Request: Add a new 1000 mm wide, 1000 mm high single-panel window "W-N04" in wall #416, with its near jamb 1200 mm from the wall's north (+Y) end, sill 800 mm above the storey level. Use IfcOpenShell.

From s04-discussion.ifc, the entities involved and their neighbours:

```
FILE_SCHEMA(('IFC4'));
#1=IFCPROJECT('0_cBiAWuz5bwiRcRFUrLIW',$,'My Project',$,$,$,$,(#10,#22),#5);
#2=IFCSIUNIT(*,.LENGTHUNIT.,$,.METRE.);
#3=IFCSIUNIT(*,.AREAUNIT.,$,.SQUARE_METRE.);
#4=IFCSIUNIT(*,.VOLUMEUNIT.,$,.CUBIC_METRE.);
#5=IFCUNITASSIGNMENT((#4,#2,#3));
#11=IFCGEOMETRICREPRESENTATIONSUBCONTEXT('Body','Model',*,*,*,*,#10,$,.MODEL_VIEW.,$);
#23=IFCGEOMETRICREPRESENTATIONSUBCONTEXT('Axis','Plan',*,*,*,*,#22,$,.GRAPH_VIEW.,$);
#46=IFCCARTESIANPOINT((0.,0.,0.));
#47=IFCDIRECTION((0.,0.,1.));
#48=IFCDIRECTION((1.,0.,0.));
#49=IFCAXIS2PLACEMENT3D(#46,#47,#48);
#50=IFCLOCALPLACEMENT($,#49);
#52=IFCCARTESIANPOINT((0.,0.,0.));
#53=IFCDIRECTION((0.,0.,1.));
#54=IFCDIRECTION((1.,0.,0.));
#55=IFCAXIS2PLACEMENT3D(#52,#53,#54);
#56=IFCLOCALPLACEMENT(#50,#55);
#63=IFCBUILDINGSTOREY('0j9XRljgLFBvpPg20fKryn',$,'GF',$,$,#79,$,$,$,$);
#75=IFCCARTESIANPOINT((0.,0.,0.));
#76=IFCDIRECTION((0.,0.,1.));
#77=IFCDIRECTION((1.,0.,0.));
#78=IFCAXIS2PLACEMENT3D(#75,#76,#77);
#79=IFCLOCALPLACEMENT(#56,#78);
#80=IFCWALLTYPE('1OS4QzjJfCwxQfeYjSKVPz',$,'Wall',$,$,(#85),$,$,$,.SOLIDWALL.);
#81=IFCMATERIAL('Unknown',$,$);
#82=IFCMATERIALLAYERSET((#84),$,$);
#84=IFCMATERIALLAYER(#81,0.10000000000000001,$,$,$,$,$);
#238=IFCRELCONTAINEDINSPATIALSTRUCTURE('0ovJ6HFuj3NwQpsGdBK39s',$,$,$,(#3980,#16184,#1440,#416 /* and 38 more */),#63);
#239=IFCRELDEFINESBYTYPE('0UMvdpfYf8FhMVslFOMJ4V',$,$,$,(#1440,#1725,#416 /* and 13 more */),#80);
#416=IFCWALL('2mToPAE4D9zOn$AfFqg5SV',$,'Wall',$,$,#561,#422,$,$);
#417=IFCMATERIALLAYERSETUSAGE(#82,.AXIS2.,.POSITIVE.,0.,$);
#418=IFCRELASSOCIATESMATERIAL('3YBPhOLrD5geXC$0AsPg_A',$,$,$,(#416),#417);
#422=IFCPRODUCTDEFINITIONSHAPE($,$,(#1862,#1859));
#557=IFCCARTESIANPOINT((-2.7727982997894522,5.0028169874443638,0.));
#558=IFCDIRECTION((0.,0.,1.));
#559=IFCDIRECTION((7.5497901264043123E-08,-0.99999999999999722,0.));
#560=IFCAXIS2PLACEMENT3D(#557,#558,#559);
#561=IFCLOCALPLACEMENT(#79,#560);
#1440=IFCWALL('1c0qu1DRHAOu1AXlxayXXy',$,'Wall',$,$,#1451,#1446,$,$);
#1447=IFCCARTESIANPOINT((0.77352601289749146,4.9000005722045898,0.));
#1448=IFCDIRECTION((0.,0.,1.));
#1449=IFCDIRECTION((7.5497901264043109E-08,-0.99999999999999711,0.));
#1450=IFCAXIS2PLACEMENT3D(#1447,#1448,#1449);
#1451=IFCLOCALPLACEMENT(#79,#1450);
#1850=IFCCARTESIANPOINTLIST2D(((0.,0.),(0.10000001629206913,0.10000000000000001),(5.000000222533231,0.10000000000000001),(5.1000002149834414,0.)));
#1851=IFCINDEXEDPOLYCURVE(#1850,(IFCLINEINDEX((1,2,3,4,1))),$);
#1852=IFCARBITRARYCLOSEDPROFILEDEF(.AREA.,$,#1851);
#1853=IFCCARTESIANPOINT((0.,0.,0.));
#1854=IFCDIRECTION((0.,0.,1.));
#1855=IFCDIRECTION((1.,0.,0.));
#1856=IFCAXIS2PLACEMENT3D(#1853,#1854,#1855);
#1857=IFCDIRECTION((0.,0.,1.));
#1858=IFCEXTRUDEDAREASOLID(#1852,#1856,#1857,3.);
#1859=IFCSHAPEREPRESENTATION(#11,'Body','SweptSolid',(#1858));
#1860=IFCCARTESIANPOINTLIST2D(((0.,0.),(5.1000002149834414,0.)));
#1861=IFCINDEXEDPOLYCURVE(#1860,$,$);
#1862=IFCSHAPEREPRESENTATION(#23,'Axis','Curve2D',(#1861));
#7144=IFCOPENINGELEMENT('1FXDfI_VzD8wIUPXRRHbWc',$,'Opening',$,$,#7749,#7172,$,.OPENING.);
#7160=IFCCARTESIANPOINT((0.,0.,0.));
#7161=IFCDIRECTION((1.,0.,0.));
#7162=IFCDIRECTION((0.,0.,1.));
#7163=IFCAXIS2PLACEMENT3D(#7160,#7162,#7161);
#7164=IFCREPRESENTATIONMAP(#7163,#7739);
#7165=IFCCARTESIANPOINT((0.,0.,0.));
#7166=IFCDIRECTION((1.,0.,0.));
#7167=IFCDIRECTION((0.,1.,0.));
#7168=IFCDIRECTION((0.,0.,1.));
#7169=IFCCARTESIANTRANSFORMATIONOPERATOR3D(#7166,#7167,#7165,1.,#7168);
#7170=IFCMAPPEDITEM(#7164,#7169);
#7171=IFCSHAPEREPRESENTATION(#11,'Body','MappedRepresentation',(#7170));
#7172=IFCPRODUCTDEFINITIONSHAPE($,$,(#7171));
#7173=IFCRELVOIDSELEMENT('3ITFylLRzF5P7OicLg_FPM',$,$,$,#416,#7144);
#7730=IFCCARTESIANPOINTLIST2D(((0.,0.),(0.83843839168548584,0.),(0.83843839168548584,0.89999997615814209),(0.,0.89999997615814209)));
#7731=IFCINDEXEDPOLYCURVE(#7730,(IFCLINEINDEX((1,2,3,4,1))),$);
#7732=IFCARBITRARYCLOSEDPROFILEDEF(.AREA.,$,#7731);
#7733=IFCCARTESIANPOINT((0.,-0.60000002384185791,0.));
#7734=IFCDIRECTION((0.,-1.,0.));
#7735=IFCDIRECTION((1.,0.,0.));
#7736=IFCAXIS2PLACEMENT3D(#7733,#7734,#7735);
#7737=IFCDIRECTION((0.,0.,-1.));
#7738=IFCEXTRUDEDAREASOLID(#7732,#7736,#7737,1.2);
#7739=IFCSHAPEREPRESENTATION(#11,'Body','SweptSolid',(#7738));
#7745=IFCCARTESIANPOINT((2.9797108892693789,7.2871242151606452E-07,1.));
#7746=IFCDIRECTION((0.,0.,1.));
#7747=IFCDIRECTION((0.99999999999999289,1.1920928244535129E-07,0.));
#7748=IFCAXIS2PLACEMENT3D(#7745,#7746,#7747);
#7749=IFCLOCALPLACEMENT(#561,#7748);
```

```python
import numpy as np
import ifcopenshell
import ifcopenshell.api.feature
import ifcopenshell.api.geometry
import ifcopenshell.api.root
import ifcopenshell.api.spatial
import ifcopenshell.geom
import ifcopenshell.util.element
import ifcopenshell.util.placement
import ifcopenshell.util.representation
import ifcopenshell.util.shape
import ifcopenshell.util.unit

model = ifcopenshell.open("s04-discussion.ifc")
unit_scale = ifcopenshell.util.unit.calculate_unit_scale(model)
settings = ifcopenshell.geom.settings()


def volume(element):
    """Net volume in cubic metres, openings subtracted."""
    shape = ifcopenshell.geom.create_shape(settings, element)
    return ifcopenshell.util.shape.get_volume(shape.geometry)


wall = model.by_guid("2mToPAE4D9zOn$AfFqg5SV")
storey = ifcopenshell.util.element.get_container(wall, ifc_class="IfcBuildingStorey")
context = ifcopenshell.util.representation.get_context(model, "Model", "Body", "MODEL_VIEW")
before = volume(wall)

width, height, from_end, sill = 1, 1, 1.2, 0.8  # metres

# The wall runs along its own X axis, and the end named is its -X end.
wall_shape = ifcopenshell.geom.create_shape(settings, wall)
x, y, z = ifcopenshell.util.shape.get_vertices(wall_shape.geometry).T
start = x.min() + from_end
face, thickness = float(y.min()), float(y.max() - y.min())
wall_matrix = ifcopenshell.util.placement.get_local_placement(wall.ObjectPlacement)
level = ifcopenshell.util.placement.get_local_placement(storey.ObjectPlacement)[2, 3]


def in_wall(x, y):
    """Placement at x, y metres in the wall's axes, at sill height."""
    matrix = wall_matrix.copy()
    matrix[:, 3] = wall_matrix @ np.array([x / unit_scale, y / unit_scale, 0.0, 1.0])
    matrix[2, 3] = level + sill / unit_scale
    return matrix


# Opening: a box that overshoots both wall faces by 50 mm.
opening = ifcopenshell.api.root.create_entity(model, ifc_class="IfcOpeningElement", predefined_type="OPENING")
box = ifcopenshell.api.geometry.add_wall_representation(
    model, context=context, length=width, height=height, thickness=thickness + 0.1
)
ifcopenshell.api.geometry.assign_representation(model, product=opening, representation=box)
ifcopenshell.api.geometry.edit_object_placement(model, product=opening, matrix=in_wall(start, face - 0.05), is_si=False)
ifcopenshell.api.feature.add_feature(model, feature=opening, element=wall)

window = ifcopenshell.api.root.create_entity(model, ifc_class="IfcWindow", name="W-N04", predefined_type="WINDOW")
window.OverallWidth, window.OverallHeight = width / unit_scale, height / unit_scale
window.PartitioningType = "SINGLE_PANEL"
body = ifcopenshell.api.geometry.add_window_representation(
    model,
    context=context,
    overall_width=window.OverallWidth,
    overall_height=window.OverallHeight,
    partition_type="SINGLE_PANEL",
)
ifcopenshell.api.geometry.assign_representation(model, product=window, representation=body)
ifcopenshell.api.spatial.assign_container(model, products=[window], relating_structure=storey)
ifcopenshell.api.feature.add_filling(model, opening=opening, element=window)

# Centre the window in the wall's thickness.
ifcopenshell.api.geometry.edit_object_placement(model, product=window, matrix=in_wall(start, face), is_si=False)
window_shape = ifcopenshell.geom.create_shape(settings, window)
depth = ifcopenshell.util.shape.get_vertices(window_shape.geometry)[:, 1]
offset = face + thickness / 2 - (depth.min() + depth.max()) / 2
ifcopenshell.api.geometry.edit_object_placement(model, product=window, matrix=in_wall(start, offset), is_si=False)

after = volume(wall)

print(f"wall volume {before:.3f} -> {after:.3f} m3")

model.write("s04-discussion_rev.ifc")
```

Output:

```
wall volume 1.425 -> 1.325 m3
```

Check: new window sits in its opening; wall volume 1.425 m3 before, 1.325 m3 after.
